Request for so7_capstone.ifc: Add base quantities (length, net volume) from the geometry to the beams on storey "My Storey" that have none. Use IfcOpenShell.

First a look at what the model holds.

```python
import ifcopenshell
import ifcopenshell.util.element
import ifcopenshell.util.unit

model = ifcopenshell.open("so7_capstone.ifc")
print(model.schema)
for unit_type in ("LENGTHUNIT", "AREAUNIT", "VOLUMEUNIT"):
    print(unit_type, ifcopenshell.util.unit.calculate_unit_scale(model, unit_type))
storey = next(s for s in model.by_type("IfcBuildingStorey") if s.Name == "My Storey")
beams = [e for e in ifcopenshell.util.element.get_decomposition(storey) if e.is_a("IfcBeam")]
for e in sorted(beams, key=lambda e: e.id()):
    print(e.id(), e.is_a(), e.Name, list(ifcopenshell.util.element.get_psets(e, qtos_only=True)), sep=" | ")
```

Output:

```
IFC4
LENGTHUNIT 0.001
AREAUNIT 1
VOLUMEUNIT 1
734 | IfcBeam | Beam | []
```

```python
import ifcopenshell
import ifcopenshell.api.pset
import ifcopenshell.geom
import ifcopenshell.util.element
import ifcopenshell.util.shape
import ifcopenshell.util.unit

model = ifcopenshell.open("so7_capstone.ifc")
unit_scale = ifcopenshell.util.unit.calculate_unit_scale(model)
volume_scale = ifcopenshell.util.unit.calculate_unit_scale(model, "VOLUMEUNIT")
settings = ifcopenshell.geom.settings()

storey = next(s for s in model.by_type("IfcBuildingStorey") if s.Name == "My Storey")
beams = [e for e in ifcopenshell.util.element.get_decomposition(storey) if e.is_a("IfcBeam")]

for e in sorted(beams, key=lambda e: e.id()):
    if ifcopenshell.util.element.get_psets(e, qtos_only=True, should_inherit=False):
        continue
    # Geometry comes back in metres, in the element's own axes.
    shape = ifcopenshell.geom.create_shape(settings, e)
    values = {
        "Length": ifcopenshell.util.shape.get_max_xyz(shape.geometry) / unit_scale,
        "NetVolume": ifcopenshell.util.shape.get_volume(shape.geometry) / volume_scale,
    }
    qto = ifcopenshell.api.pset.add_qto(model, product=e, name="Qto_BeamBaseQuantities")
    ifcopenshell.api.pset.edit_qto(model, qto=qto, properties=values)
    print(e.id(), {k: round(v, 3) for k, v in values.items()})

model.write("so7_capstone-out.ifc")
```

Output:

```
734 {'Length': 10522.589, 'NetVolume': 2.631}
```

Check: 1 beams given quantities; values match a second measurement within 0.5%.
